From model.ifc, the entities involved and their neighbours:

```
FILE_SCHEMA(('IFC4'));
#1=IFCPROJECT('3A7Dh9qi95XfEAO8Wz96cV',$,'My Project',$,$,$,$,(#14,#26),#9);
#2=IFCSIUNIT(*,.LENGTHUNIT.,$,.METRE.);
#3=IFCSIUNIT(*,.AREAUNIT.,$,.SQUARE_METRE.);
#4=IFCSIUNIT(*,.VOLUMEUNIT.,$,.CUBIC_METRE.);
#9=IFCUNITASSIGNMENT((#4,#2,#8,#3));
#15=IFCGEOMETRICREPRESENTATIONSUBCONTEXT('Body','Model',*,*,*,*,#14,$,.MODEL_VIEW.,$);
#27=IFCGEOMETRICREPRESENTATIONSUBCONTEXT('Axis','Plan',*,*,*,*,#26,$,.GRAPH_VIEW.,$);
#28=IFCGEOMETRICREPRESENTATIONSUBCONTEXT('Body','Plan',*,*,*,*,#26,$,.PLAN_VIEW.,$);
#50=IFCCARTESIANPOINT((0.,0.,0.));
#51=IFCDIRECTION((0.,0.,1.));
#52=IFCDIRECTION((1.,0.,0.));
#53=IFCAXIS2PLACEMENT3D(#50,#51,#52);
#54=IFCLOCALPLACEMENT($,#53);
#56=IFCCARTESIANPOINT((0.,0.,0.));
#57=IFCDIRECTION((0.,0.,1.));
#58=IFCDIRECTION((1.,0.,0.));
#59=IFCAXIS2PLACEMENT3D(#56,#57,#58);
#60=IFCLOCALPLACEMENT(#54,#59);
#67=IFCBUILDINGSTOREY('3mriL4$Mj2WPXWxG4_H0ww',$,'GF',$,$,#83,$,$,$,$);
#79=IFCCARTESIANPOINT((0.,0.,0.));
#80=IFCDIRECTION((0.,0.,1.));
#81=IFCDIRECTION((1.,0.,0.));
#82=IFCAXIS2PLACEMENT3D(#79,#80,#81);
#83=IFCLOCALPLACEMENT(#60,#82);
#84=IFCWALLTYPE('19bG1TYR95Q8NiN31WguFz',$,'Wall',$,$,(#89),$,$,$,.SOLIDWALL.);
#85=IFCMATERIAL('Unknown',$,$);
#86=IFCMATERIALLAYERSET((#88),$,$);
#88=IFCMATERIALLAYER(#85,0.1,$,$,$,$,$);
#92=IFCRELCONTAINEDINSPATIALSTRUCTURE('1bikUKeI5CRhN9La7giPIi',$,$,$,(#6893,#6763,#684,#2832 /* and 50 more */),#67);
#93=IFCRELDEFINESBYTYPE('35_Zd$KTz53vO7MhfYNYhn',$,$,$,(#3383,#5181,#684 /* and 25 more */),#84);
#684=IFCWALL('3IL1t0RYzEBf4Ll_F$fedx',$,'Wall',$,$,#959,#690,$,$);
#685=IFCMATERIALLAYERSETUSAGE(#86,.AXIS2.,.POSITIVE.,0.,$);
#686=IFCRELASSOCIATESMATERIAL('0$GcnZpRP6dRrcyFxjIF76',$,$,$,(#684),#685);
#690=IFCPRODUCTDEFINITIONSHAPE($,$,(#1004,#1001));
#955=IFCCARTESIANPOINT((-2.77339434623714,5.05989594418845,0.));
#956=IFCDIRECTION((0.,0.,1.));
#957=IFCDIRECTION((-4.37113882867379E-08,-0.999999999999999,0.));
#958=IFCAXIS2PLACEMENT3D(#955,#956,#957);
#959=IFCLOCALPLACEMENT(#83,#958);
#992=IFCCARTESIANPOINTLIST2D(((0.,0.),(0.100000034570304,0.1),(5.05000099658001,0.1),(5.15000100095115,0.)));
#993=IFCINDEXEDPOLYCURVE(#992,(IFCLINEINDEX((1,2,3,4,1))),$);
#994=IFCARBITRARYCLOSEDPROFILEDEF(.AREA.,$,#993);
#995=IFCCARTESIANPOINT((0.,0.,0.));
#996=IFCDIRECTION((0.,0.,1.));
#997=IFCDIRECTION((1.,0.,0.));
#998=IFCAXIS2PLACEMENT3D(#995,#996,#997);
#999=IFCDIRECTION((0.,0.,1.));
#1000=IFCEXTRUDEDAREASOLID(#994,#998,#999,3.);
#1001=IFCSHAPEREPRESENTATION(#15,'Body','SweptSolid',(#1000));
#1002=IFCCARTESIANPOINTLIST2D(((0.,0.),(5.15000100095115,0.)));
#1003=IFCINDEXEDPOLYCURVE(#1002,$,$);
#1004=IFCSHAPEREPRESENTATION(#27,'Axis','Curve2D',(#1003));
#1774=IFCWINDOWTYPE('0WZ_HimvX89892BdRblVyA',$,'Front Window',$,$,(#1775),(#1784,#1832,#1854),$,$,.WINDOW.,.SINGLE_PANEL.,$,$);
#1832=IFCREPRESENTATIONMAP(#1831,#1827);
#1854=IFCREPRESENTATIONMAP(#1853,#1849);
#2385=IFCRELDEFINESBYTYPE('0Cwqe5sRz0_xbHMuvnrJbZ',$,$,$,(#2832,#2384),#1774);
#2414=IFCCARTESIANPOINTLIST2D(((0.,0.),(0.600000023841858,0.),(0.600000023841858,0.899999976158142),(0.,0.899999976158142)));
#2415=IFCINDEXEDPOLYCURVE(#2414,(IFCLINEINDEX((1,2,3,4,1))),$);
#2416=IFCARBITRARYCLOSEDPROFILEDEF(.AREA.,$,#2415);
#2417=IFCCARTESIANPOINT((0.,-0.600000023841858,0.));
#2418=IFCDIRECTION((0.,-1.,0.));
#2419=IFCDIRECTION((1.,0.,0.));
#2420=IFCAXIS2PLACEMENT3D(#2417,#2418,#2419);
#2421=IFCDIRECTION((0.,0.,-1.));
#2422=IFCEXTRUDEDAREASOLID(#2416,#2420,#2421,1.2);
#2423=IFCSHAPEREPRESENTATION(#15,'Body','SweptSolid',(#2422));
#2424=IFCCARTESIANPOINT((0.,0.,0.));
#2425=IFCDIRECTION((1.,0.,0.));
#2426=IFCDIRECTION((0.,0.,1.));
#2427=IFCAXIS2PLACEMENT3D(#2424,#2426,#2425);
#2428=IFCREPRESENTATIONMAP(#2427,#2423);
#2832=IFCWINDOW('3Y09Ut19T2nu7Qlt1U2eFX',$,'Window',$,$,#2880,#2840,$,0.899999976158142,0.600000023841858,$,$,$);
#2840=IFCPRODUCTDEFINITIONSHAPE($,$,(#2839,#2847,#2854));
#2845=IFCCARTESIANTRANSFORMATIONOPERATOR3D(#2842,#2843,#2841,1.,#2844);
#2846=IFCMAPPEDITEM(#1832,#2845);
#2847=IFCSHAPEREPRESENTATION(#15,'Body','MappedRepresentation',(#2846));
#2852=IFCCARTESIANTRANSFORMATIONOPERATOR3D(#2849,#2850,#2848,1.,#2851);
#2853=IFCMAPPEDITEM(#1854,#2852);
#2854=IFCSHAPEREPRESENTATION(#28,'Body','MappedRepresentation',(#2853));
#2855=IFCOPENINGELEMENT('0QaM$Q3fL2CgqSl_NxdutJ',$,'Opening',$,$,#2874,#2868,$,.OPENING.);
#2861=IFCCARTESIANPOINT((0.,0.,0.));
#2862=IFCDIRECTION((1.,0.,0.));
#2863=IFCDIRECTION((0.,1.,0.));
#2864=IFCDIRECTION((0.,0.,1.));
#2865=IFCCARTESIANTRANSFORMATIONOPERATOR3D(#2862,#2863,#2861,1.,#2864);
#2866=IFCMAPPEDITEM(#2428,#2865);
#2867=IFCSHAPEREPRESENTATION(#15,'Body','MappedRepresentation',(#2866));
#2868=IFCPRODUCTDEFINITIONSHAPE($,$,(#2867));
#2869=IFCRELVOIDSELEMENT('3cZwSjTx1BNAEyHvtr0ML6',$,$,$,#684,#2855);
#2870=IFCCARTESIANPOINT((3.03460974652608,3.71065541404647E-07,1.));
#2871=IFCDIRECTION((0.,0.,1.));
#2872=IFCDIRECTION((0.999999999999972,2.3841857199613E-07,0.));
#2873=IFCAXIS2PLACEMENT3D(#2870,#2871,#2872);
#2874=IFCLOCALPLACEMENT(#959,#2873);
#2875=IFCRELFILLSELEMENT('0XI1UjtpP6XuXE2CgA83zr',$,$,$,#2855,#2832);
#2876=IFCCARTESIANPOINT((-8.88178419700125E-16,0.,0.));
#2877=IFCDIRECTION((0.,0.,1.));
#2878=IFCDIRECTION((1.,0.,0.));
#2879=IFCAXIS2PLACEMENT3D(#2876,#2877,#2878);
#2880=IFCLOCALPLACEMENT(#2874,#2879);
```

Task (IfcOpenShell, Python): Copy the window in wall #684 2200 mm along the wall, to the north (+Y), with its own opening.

```python
import ifcopenshell
import ifcopenshell.api.feature
import ifcopenshell.api.geometry
import ifcopenshell.api.root
import ifcopenshell.geom
import ifcopenshell.util.element
import ifcopenshell.util.placement
import ifcopenshell.util.shape

model = ifcopenshell.open("model.ifc")
settings = ifcopenshell.geom.settings()


def volume(element):
    """Net volume in cubic metres, openings subtracted."""
    shape = ifcopenshell.geom.create_shape(settings, element)
    return ifcopenshell.util.shape.get_volume(shape.geometry)


window = model.by_id(2832)
opening = window.FillsVoids[0].RelatingOpeningElement
wall = opening.VoidsElements[0].RelatingBuildingElement
before = volume(wall)
shift = ifcopenshell.util.placement.get_local_placement(wall.ObjectPlacement)[:3, 0] * -2.2

# copy_class copies the void relationship, type, container and properties, but no geometry.
new_opening = ifcopenshell.api.root.copy_class(model, product=opening)
new_opening.Representation = ifcopenshell.util.element.copy_deep(
    model, opening.Representation, exclude=["IfcGeometricRepresentationContext", "IfcRepresentationMap"]
)
new_window = ifcopenshell.api.root.copy_class(model, product=window)
new_window.Representation = ifcopenshell.util.element.copy_deep(
    model, window.Representation, exclude=["IfcGeometricRepresentationContext", "IfcRepresentationMap"]
)
ifcopenshell.api.feature.add_filling(model, opening=new_opening, element=new_window)

for old, new in ((opening, new_opening), (window, new_window)):
    matrix = ifcopenshell.util.placement.get_local_placement(old.ObjectPlacement)
    matrix[:3, 3] += shift
    ifcopenshell.api.geometry.edit_object_placement(model, product=new, matrix=matrix, is_si=False)

after = volume(wall)

print(f"wall volume {before:.3f} -> {after:.3f} m3")

model.write("model_v2.ifc")
```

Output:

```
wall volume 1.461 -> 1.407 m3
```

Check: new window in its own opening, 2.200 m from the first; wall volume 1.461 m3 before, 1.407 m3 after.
